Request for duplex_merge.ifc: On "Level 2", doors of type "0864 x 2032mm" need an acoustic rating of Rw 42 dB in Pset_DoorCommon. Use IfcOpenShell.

First a look at what the model holds.

```python
import ifcopenshell
import ifcopenshell.util.element

model = ifcopenshell.open("duplex_merge.ifc")
print(model.schema)
storey = next(s for s in model.by_type("IfcBuildingStorey") if s.Name == "Level 2")
doors = [e for e in ifcopenshell.util.element.get_decomposition(storey) if e.is_a("IfcDoor")]
seen = {}
for e in doors:
    element_type = ifcopenshell.util.element.get_type(e)
    key = (element_type.Name if element_type != e and element_type else None, ifcopenshell.util.element.get_pset(e, "Pset_DoorCommon", "AcousticRating"))
    seen[key] = seen.get(key, 0) + 1
for (name, value), count in sorted(seen.items(), key=str):
    print(count, "x", name, "|", value)
```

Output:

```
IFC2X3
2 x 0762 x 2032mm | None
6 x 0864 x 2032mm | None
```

```python
import ifcopenshell
import ifcopenshell.api.pset
import ifcopenshell.util.element

model = ifcopenshell.open("duplex_merge.ifc")

storey = next(s for s in model.by_type("IfcBuildingStorey") if s.Name == "Level 2")
doors = [e for e in ifcopenshell.util.element.get_decomposition(storey) if e.is_a("IfcDoor")]

count = 0
for e in doors:
    element_type = ifcopenshell.util.element.get_type(e)
    if element_type in (None, e) or element_type.Name != "0864 x 2032mm":
        continue
    # add_pset returns the element's existing set when there is one.
    pset = ifcopenshell.api.pset.add_pset(model, product=e, name="Pset_DoorCommon")
    ifcopenshell.api.pset.edit_pset(model, pset=pset, properties={"AcousticRating": "Rw 42 dB"})
    count += 1

print(count, "doors updated")

model.write("duplex_merge_updated.ifc")
```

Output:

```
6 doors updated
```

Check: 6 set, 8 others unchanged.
